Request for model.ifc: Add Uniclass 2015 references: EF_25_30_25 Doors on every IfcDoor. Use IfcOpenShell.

First a look at what the model holds.

```python
import ifcopenshell

model = ifcopenshell.open("model.ifc")
print(model.schema)
print("classifications:", [c.Name for c in model.by_type("IfcClassification")])
for ifc_class in ("IfcDoor", "IfcRoof", "IfcStair", "IfcWall", "IfcWindow"):
    print(ifc_class, len(model.by_type(ifc_class)))
```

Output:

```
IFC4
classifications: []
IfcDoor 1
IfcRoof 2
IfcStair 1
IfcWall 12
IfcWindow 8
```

```python
import ifcopenshell
import ifcopenshell.api.classification

model = ifcopenshell.open("model.ifc")

system = ifcopenshell.api.classification.add_classification(model, classification="Uniclass 2015")

codes = {
    "IfcDoor": ("EF_25_30_25", "Doors"),
}
for ifc_class, (code, name) in codes.items():
    products = model.by_type(ifc_class)
    ifcopenshell.api.classification.add_reference(
        model, products=products, classification=system, identification=code, name=name
    )
    print(code, len(products))

model.write("model_rev.ifc")
```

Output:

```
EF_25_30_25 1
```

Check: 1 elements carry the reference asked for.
